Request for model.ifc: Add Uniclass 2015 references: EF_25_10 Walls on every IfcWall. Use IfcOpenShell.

First a look at what the model holds.

```python
import ifcopenshell

model = ifcopenshell.open("model.ifc")
print(model.schema)
print("classifications:", [c.Name for c in model.by_type("IfcClassification")])
for ifc_class in ("IfcDoor", "IfcRoof", "IfcStair", "IfcWall", "IfcWindow"):
    print(ifc_class, len(model.by_type(ifc_class)))
```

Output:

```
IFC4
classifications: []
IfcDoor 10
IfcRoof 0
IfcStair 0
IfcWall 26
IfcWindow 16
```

```python
import ifcopenshell
import ifcopenshell.api.classification

model = ifcopenshell.open("model.ifc")

system = ifcopenshell.api.classification.add_classification(model, classification="Uniclass 2015")

codes = {
    "IfcWall": ("EF_25_10", "Walls"),
}
for ifc_class, (code, name) in codes.items():
    products = model.by_type(ifc_class)
    ifcopenshell.api.classification.add_reference(
        model, products=products, classification=system, identification=code, name=name
    )
    print(code, len(products))

model.write("model_edited.ifc")
```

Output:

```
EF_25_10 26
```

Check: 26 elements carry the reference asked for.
